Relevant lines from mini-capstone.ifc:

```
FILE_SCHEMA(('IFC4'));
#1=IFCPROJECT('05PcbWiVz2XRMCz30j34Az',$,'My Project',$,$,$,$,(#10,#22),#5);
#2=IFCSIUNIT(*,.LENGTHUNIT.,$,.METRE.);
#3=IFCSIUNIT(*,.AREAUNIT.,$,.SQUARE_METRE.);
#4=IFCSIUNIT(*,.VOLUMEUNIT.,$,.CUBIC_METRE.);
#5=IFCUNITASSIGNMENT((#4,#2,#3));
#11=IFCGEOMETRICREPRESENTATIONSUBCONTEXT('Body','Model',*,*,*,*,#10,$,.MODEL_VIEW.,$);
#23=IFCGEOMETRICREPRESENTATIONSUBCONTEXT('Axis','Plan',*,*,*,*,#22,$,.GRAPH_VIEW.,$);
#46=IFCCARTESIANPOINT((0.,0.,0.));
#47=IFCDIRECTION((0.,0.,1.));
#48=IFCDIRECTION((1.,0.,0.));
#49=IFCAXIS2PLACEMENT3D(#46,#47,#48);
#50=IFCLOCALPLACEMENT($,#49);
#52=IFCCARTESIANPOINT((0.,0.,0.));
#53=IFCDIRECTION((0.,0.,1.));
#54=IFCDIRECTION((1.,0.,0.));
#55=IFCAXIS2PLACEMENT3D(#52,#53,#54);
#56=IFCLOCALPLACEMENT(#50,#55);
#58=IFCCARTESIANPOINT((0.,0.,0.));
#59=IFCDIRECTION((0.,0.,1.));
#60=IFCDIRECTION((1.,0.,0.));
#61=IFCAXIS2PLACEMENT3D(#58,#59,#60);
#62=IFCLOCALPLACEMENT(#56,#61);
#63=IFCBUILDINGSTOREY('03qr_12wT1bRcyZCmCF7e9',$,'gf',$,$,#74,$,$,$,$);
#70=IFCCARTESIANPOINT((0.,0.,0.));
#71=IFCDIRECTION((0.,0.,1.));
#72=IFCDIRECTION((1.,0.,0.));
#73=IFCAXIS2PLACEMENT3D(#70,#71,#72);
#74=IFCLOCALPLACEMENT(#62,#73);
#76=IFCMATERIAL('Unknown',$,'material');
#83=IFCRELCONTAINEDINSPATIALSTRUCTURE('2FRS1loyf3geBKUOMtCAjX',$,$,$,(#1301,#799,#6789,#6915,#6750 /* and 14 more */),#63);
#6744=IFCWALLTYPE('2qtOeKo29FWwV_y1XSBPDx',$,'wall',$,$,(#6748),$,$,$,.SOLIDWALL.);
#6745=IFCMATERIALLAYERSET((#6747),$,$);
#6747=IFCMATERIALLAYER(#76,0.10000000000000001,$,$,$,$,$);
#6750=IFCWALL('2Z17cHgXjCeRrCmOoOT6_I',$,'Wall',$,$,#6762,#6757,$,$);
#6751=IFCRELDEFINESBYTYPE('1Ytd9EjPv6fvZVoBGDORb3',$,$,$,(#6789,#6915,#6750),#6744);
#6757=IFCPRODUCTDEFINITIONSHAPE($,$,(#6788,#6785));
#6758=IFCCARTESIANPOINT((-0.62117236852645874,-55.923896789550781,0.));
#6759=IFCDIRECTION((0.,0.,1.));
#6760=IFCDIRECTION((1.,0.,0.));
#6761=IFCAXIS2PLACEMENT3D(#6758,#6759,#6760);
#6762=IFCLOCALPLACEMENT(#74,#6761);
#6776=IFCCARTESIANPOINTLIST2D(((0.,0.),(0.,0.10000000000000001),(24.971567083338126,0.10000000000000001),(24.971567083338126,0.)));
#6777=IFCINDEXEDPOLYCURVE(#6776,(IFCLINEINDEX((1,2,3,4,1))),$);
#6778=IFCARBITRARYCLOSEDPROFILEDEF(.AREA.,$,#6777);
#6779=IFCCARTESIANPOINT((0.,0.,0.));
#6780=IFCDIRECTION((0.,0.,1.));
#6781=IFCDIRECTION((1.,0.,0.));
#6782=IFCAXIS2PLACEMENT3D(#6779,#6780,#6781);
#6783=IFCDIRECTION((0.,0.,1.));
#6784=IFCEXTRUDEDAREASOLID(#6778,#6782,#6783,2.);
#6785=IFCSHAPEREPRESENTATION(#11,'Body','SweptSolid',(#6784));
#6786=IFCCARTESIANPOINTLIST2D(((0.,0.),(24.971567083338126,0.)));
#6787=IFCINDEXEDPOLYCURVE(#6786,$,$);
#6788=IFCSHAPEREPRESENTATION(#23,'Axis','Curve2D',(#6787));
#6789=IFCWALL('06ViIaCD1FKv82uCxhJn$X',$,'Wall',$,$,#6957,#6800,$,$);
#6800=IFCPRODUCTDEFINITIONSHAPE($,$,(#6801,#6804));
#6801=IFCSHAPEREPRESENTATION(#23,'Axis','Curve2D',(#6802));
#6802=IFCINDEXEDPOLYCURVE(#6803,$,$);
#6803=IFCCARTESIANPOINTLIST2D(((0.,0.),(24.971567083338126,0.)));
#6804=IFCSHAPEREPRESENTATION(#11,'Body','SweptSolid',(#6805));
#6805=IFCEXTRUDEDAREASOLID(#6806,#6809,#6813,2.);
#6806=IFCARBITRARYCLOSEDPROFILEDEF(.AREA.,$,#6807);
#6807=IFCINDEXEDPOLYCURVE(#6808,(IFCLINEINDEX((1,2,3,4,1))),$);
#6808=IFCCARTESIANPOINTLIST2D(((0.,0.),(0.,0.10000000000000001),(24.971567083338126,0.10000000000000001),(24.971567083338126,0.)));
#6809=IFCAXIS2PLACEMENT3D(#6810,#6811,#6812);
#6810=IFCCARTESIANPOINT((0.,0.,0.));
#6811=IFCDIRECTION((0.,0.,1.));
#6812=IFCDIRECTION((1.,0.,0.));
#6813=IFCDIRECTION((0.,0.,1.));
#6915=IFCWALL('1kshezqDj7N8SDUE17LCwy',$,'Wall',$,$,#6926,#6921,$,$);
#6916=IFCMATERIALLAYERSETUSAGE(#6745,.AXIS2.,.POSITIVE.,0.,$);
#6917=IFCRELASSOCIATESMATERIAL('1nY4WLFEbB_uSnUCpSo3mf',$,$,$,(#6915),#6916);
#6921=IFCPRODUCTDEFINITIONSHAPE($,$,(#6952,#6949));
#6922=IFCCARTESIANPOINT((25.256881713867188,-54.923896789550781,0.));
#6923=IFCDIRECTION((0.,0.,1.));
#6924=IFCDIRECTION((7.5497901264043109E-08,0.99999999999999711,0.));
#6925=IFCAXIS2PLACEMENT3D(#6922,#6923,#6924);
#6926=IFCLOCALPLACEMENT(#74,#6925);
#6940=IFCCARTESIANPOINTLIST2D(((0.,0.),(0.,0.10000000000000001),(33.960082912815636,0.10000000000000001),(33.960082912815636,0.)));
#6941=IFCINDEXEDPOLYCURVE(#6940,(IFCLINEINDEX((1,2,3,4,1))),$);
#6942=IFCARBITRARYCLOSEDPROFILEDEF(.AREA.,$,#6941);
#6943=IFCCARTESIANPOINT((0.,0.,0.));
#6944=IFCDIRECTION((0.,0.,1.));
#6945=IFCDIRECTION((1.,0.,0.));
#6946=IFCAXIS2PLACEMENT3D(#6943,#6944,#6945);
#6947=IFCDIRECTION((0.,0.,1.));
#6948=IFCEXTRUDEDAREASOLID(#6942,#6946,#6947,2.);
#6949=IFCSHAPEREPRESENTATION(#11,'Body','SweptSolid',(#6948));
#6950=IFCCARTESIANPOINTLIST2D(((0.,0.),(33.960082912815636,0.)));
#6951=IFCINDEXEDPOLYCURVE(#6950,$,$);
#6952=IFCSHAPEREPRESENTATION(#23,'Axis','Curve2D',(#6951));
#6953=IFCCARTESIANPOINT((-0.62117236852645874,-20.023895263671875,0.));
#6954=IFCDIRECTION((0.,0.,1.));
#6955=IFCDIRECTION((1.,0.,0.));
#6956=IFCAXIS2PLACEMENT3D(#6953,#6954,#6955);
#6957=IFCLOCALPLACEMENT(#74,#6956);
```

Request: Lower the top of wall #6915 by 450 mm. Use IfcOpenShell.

```python
import ifcopenshell
import ifcopenshell.geom
import ifcopenshell.util.representation
import ifcopenshell.util.shape
import ifcopenshell.util.unit

model = ifcopenshell.open("mini-capstone.ifc")
unit_scale = ifcopenshell.util.unit.calculate_unit_scale(model)
settings = ifcopenshell.geom.settings()


def volume(element):
    """Net volume in cubic metres, openings subtracted."""
    shape = ifcopenshell.geom.create_shape(settings, element)
    return ifcopenshell.util.shape.get_volume(shape.geometry)


wall = model.by_guid("1kshezqDj7N8SDUE17LCwy")
before = volume(wall)

body = ifcopenshell.util.representation.get_representation(wall, "Model", "Body")
solid = body.Items[0]
old_height = solid.Depth
solid.Depth -= 0.45 / unit_scale
after = volume(wall)

print(f"height {old_height:g} -> {solid.Depth:g}, volume {before:.3f} -> {after:.3f} m3")

model.write("mini-capstone_rev.ifc")
```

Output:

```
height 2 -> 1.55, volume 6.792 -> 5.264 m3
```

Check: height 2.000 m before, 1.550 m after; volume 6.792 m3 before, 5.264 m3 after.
